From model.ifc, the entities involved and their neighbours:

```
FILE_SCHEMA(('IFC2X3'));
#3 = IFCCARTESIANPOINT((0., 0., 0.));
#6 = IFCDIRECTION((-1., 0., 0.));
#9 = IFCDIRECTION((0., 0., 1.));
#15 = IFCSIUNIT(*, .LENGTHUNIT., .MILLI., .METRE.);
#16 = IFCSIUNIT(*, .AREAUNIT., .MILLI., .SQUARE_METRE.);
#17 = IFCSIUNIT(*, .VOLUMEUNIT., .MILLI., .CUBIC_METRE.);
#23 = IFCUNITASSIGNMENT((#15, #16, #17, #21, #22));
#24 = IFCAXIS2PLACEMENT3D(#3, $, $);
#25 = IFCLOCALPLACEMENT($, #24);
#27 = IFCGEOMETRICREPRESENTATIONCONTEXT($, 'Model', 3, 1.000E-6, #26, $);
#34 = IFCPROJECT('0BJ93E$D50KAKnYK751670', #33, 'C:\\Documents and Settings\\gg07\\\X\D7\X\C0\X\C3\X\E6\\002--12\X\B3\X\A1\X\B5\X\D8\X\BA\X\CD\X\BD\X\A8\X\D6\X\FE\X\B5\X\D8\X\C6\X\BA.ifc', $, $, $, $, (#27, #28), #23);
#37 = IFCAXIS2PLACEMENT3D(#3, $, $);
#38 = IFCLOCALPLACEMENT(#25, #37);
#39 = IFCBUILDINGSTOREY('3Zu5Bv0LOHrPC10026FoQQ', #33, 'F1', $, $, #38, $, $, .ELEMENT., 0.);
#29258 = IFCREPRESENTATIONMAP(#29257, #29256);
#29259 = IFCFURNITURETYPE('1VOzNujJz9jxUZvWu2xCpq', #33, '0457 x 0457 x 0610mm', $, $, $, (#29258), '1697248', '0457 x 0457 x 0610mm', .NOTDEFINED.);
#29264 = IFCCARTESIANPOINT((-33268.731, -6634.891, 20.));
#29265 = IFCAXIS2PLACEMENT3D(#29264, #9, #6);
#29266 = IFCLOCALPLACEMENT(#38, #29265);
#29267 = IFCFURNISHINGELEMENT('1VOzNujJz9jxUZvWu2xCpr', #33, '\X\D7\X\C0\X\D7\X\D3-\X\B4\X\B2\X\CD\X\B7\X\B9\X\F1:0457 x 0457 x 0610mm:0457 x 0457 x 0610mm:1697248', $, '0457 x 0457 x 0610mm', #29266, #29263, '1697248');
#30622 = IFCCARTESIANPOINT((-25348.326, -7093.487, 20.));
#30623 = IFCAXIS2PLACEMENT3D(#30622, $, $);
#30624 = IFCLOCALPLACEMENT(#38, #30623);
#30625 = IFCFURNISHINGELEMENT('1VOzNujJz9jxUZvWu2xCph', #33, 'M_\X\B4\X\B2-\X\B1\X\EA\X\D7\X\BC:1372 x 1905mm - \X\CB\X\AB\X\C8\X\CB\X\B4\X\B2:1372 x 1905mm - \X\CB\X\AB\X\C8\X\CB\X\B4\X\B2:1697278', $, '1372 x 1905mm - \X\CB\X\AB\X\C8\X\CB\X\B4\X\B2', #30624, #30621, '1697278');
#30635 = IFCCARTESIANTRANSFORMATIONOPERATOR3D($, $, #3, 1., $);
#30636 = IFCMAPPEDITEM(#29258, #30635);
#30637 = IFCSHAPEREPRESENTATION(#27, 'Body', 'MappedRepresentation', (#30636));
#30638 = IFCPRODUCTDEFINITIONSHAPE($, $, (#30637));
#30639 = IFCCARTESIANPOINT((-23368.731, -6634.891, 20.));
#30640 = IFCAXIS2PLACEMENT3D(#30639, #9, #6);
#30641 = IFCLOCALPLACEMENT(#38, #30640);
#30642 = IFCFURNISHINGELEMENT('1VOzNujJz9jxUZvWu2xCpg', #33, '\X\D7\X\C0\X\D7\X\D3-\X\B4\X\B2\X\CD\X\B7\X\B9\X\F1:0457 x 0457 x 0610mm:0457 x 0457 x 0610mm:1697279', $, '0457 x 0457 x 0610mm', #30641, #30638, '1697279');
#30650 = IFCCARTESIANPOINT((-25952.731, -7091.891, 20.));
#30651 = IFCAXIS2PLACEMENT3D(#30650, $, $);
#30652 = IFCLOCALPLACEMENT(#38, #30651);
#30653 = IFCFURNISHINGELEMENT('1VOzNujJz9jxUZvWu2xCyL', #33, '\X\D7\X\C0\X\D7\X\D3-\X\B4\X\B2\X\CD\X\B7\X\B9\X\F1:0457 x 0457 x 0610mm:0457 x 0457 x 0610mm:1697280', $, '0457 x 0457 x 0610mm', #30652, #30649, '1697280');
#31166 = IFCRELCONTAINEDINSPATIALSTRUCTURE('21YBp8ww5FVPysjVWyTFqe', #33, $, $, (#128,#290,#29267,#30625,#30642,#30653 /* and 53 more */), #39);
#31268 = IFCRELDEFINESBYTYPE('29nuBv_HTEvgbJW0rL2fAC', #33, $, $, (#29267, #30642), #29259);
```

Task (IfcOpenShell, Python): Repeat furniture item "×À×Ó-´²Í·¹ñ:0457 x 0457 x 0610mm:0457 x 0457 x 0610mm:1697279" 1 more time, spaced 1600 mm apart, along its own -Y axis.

```python
import ifcopenshell
import ifcopenshell.api.geometry
import ifcopenshell.api.root
import ifcopenshell.util.element
import ifcopenshell.util.placement
import ifcopenshell.util.unit

model = ifcopenshell.open("model.ifc")
unit_scale = ifcopenshell.util.unit.calculate_unit_scale(model)


def reuse_history(source, copy):
    """copy_class also copies each property set's owner history, people and application; keep the originals."""
    for rel in copy.IsDefinedBy:
        if rel.is_a("IfcRelDefinesByProperties") and (history := rel.RelatingPropertyDefinition.OwnerHistory):
            rel.RelatingPropertyDefinition.OwnerHistory = source.OwnerHistory
            ifcopenshell.util.element.remove_deep2(model, history)


source = model.by_guid("1VOzNujJz9jxUZvWu2xCpg")
base = ifcopenshell.util.placement.get_local_placement(source.ObjectPlacement)
step = -base[:3, 1] * 1.6 / unit_scale

for i in range(1, 2):
    copy = ifcopenshell.api.root.copy_class(model, product=source)
    copy.Representation = ifcopenshell.util.element.copy_deep(
        model, source.Representation, exclude=["IfcGeometricRepresentationContext", "IfcRepresentationMap"]
    )
    copy.Name = "×À×Ó-´²Í·¹ñ:0457 x 0457 x 0610mm:0457 x 0457 x 0610mm"
    copy.Tag = None
    reuse_history(source, copy)
    matrix = base.copy()
    matrix[:3, 3] += i * step
    print("added at", matrix[:3, 3].round(3) + 0.0)
    ifcopenshell.api.geometry.edit_object_placement(model, product=copy, matrix=matrix, is_si=False)

model.write("model_v2.ifc")
```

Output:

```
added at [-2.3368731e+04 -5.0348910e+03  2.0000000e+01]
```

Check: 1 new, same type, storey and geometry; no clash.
